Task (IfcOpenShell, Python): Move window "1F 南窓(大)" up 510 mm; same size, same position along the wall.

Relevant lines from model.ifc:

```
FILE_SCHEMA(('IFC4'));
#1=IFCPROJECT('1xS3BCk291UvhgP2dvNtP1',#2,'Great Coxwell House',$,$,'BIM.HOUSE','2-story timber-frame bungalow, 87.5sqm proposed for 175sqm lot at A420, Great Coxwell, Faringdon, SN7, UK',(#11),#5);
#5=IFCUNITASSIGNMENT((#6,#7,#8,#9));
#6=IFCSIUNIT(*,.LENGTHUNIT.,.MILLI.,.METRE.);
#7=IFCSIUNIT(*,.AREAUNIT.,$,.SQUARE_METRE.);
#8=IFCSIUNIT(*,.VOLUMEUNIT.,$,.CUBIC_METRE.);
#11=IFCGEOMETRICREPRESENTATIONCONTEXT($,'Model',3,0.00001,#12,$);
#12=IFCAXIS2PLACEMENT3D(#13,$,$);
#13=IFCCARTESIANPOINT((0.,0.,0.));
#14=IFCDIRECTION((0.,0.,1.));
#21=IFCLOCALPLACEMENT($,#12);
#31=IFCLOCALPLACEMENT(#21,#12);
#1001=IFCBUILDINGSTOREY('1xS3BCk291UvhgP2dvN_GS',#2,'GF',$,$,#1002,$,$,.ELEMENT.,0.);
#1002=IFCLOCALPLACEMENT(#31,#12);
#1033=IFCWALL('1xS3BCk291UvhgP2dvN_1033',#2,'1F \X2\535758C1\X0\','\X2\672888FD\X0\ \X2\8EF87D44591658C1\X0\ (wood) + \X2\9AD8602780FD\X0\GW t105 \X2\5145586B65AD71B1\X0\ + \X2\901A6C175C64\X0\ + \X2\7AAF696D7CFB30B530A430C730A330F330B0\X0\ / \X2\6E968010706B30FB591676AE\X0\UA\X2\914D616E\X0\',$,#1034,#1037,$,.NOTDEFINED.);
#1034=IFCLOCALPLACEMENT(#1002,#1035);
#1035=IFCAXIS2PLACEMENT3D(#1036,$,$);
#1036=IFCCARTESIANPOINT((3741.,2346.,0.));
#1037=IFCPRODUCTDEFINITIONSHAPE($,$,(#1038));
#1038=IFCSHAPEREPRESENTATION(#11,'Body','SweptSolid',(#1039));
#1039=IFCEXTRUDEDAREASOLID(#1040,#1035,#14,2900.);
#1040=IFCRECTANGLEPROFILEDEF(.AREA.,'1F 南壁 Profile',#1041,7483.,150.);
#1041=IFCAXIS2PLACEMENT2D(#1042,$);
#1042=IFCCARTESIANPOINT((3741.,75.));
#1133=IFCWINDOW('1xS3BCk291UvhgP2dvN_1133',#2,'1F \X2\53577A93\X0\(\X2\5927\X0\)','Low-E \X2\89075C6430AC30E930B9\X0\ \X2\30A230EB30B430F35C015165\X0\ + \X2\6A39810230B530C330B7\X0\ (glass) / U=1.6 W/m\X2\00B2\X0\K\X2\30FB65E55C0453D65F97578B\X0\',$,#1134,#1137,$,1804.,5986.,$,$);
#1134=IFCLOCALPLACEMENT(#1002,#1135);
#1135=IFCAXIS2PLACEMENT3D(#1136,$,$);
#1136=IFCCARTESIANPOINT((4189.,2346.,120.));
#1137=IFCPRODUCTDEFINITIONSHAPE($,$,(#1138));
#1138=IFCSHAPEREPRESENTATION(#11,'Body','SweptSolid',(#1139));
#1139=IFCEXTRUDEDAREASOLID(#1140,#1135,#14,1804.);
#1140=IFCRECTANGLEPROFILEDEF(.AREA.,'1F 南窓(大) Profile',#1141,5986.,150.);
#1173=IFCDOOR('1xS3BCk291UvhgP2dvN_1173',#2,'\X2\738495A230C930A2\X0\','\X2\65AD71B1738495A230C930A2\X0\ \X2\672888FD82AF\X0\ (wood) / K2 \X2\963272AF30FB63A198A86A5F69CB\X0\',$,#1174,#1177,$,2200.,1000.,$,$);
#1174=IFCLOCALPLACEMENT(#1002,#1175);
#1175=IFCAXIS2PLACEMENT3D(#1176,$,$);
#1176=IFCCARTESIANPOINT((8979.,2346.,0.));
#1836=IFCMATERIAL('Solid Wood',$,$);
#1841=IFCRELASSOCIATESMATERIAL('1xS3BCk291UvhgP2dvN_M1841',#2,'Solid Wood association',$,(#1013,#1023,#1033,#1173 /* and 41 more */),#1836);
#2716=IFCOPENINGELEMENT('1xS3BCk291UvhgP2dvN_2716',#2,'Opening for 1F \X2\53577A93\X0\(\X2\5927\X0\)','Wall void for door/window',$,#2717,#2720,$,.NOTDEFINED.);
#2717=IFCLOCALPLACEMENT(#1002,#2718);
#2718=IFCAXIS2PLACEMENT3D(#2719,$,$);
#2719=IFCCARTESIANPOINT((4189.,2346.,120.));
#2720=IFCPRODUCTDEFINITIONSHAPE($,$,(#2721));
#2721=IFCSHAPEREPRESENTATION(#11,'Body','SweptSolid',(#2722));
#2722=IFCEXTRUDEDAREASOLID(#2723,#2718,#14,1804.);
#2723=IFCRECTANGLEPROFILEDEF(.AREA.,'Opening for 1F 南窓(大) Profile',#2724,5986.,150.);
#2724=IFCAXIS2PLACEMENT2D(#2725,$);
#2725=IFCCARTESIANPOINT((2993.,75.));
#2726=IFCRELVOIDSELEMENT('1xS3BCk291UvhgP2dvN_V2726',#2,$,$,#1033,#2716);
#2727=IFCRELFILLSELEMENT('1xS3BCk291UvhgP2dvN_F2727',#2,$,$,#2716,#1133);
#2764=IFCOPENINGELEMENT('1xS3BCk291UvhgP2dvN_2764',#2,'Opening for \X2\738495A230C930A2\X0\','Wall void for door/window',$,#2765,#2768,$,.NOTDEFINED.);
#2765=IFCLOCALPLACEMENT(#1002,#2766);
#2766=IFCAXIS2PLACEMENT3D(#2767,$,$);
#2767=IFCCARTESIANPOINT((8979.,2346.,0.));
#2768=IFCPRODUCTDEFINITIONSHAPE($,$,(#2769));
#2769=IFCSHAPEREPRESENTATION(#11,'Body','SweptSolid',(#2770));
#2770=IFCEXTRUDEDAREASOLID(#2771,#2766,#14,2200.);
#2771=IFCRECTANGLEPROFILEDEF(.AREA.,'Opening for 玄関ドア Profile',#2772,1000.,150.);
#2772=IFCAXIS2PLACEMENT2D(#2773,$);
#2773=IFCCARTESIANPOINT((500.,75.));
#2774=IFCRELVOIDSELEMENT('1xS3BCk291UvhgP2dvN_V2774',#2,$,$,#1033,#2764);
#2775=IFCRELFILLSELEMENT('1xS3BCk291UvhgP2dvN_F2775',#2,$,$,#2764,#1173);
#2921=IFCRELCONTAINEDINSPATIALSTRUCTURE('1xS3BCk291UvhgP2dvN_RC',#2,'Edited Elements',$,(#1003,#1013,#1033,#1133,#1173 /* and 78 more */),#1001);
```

```python
import numpy as np
import ifcopenshell
import ifcopenshell.api.geometry
import ifcopenshell.util.placement
import ifcopenshell.util.unit

model = ifcopenshell.open("model.ifc")
unit_scale = ifcopenshell.util.unit.calculate_unit_scale(model)

window = model.by_id(1133)
opening = window.FillsVoids[0].RelatingOpeningElement
dz = 0.51 / unit_scale

shift = np.array([0.0, 0.0, dz])
# The window is not placed relative to its opening, so move both.
for product in (opening, window):
    matrix = ifcopenshell.util.placement.get_local_placement(product.ObjectPlacement)
    matrix[:3, 3] += shift
    ifcopenshell.api.geometry.edit_object_placement(model, product=product, matrix=matrix, is_si=False)

print(f"moved by {dz * unit_scale:+.3f} m")

model.write("model_v2.ifc")
```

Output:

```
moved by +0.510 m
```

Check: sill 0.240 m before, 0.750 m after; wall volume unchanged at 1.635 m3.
